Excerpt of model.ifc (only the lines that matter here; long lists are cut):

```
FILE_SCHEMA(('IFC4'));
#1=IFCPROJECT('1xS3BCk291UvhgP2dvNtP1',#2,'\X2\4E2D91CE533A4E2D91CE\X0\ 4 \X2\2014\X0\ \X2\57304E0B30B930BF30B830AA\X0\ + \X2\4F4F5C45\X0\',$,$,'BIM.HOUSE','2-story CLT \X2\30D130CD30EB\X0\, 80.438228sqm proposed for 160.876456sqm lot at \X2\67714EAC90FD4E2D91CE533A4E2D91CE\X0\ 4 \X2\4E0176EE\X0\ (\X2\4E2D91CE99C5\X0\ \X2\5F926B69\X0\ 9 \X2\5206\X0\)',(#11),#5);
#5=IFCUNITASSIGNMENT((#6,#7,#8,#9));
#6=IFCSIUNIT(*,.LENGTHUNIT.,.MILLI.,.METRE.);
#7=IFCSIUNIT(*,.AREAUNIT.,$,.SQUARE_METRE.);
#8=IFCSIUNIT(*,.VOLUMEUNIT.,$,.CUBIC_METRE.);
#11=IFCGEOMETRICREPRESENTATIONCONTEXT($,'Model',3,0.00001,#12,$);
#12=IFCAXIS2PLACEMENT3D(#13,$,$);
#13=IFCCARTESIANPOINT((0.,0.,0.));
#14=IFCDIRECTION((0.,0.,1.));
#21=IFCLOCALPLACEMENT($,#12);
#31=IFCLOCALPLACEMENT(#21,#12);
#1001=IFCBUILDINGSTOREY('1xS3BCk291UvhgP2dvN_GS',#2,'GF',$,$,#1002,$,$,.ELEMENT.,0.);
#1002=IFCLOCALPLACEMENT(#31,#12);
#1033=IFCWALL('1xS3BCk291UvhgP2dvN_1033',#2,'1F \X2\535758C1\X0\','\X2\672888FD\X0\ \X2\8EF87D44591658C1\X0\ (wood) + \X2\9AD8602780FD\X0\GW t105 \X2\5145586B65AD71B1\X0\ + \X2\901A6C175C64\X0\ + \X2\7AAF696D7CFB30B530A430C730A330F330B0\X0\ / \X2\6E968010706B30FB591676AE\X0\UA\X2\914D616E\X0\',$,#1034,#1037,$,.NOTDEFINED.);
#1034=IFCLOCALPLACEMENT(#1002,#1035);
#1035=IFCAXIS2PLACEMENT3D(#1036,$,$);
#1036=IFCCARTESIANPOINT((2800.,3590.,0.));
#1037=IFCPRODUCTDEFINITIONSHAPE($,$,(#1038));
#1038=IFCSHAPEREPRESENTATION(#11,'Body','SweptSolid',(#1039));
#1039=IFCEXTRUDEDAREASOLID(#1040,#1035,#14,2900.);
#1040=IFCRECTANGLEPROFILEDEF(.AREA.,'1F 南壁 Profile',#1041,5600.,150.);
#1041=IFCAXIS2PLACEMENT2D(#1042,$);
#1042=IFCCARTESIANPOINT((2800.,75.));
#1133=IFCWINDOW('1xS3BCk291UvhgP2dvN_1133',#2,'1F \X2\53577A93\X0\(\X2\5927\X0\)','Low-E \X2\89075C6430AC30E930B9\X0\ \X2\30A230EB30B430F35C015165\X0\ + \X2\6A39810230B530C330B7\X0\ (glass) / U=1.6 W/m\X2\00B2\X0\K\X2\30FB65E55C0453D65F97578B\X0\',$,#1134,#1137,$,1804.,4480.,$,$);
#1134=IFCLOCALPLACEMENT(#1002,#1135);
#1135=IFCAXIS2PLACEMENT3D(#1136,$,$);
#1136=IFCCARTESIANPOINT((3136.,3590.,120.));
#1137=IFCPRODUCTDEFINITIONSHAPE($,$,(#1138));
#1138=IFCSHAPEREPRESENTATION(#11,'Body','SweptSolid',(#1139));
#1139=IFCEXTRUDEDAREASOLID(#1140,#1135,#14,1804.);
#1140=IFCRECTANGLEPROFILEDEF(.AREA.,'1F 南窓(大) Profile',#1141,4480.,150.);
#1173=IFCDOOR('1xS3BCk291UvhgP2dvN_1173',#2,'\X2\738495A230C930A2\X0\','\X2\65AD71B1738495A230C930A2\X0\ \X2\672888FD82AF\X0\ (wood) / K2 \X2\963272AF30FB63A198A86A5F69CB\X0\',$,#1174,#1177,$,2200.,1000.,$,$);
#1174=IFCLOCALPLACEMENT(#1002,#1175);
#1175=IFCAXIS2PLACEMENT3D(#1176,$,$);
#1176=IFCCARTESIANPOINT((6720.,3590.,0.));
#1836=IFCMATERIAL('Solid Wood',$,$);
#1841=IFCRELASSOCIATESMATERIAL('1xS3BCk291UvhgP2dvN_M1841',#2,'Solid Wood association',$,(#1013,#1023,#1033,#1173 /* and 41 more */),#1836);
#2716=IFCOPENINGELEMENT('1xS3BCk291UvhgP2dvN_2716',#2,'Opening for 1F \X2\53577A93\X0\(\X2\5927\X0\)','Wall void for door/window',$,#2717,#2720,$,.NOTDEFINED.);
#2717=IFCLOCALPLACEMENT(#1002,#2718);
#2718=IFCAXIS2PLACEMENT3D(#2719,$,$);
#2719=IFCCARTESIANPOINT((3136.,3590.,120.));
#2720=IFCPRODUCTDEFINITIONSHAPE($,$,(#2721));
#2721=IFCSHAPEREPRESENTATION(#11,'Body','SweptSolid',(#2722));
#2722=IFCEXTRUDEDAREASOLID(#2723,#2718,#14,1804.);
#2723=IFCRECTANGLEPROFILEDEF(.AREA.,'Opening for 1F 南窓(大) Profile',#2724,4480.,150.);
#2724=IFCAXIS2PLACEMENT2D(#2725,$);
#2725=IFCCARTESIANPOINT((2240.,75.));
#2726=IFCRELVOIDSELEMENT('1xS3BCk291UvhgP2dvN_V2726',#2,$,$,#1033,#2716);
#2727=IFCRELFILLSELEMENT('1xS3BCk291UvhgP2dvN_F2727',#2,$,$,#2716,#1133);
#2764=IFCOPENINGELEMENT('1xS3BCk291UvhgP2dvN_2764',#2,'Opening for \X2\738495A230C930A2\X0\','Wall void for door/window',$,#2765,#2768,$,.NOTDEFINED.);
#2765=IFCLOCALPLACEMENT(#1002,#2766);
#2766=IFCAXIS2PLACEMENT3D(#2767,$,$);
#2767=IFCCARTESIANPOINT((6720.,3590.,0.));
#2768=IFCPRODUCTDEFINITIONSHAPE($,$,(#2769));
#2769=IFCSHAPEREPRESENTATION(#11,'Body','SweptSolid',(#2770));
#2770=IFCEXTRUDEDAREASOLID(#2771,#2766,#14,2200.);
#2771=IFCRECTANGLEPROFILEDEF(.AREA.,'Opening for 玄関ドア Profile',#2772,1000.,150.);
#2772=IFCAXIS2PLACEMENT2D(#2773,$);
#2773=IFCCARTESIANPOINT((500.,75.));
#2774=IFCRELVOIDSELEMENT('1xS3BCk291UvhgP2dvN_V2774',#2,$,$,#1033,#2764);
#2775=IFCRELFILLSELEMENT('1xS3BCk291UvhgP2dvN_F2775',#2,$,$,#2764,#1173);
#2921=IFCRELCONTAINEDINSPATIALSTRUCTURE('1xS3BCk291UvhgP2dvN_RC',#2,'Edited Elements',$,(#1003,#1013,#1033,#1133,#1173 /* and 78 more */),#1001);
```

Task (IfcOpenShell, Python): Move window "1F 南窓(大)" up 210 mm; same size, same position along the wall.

```python
import numpy as np
import ifcopenshell
import ifcopenshell.api.geometry
import ifcopenshell.util.placement
import ifcopenshell.util.unit

model = ifcopenshell.open("model.ifc")
unit_scale = ifcopenshell.util.unit.calculate_unit_scale(model)

window = model.by_id(1133)
opening = window.FillsVoids[0].RelatingOpeningElement
dz = 0.21 / unit_scale

shift = np.array([0.0, 0.0, dz])
# The window is not placed relative to its opening, so move both.
for product in (opening, window):
    matrix = ifcopenshell.util.placement.get_local_placement(product.ObjectPlacement)
    matrix[:3, 3] += shift
    ifcopenshell.api.geometry.edit_object_placement(model, product=product, matrix=matrix, is_si=False)

print(f"moved by {dz * unit_scale:+.3f} m")

model.write("model-out.ifc")
```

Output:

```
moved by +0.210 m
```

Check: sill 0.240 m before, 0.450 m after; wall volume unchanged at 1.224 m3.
